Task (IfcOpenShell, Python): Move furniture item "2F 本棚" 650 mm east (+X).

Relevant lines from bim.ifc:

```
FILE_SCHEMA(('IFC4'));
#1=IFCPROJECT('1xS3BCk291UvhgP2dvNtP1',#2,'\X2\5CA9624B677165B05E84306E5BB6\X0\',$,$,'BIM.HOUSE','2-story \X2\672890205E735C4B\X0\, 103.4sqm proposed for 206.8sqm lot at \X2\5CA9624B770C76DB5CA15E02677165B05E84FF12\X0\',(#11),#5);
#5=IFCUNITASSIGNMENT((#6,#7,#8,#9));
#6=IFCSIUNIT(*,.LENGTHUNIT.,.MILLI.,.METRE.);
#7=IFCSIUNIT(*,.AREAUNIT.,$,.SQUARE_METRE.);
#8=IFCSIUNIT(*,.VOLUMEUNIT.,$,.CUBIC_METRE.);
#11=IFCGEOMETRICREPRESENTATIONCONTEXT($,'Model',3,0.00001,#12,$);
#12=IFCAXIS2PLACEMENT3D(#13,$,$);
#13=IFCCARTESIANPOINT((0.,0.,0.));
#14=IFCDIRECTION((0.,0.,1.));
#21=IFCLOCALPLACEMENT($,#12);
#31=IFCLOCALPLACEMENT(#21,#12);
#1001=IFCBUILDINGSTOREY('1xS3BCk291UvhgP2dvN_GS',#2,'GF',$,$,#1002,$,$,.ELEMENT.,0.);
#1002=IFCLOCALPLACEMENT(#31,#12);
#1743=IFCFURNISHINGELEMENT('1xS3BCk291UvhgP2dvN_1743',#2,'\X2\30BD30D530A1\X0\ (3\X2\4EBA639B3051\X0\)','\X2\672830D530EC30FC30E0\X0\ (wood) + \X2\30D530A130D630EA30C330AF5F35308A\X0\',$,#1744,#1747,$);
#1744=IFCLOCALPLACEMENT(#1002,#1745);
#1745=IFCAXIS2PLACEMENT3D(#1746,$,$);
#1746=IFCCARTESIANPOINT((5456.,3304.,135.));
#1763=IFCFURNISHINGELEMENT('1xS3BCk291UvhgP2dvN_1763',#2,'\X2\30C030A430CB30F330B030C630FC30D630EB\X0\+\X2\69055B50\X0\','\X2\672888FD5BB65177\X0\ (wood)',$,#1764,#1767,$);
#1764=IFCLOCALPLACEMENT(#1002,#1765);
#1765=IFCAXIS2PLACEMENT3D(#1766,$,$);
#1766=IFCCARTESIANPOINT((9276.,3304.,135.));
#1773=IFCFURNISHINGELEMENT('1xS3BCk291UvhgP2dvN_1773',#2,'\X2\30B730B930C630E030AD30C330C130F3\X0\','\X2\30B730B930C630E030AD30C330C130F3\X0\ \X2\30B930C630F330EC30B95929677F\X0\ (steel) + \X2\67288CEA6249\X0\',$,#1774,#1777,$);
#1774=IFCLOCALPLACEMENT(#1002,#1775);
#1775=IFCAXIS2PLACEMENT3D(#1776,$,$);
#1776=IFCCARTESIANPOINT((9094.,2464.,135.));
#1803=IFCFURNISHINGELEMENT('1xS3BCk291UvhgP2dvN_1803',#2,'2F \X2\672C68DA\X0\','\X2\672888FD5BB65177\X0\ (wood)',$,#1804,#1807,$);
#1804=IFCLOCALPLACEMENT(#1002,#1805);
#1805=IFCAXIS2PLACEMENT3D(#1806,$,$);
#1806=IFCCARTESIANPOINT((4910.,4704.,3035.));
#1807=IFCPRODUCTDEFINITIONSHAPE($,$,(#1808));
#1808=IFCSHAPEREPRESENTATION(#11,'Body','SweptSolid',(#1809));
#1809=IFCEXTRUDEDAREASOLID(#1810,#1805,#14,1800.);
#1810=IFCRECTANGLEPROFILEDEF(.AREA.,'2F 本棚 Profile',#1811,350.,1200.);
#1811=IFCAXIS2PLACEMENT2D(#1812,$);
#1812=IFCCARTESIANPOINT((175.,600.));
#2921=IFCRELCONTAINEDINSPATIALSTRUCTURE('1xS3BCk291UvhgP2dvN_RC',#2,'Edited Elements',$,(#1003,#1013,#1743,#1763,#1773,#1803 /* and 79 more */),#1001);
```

```python
import ifcopenshell
import ifcopenshell.api.geometry
import ifcopenshell.util.placement
import ifcopenshell.util.unit

model = ifcopenshell.open("bim.ifc")
unit_scale = ifcopenshell.util.unit.calculate_unit_scale(model)

item = model.by_guid("1xS3BCk291UvhgP2dvN_1803")
matrix = ifcopenshell.util.placement.get_local_placement(item.ObjectPlacement)
matrix[0, 3] += 0.65 / unit_scale
ifcopenshell.api.geometry.edit_object_placement(model, product=item, matrix=matrix, is_si=False)

print(ifcopenshell.util.placement.get_local_placement(item.ObjectPlacement).round(3) + 0.0)

model.write("bim_updated.ifc")
```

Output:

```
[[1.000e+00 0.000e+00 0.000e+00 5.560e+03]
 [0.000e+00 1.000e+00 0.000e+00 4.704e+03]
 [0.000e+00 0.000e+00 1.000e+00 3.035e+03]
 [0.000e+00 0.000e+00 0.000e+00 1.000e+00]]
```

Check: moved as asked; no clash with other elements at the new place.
